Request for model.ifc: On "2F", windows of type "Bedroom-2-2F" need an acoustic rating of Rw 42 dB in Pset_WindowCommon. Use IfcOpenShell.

First a look at what the model holds.

```python
import ifcopenshell
import ifcopenshell.util.element

model = ifcopenshell.open("model.ifc")
print(model.schema)
storey = next(s for s in model.by_type("IfcBuildingStorey") if s.Name == "2F")
windows = [e for e in ifcopenshell.util.element.get_decomposition(storey) if e.is_a("IfcWindow")]
seen = {}
for e in windows:
    element_type = ifcopenshell.util.element.get_type(e)
    key = (element_type.Name if element_type != e and element_type else None, ifcopenshell.util.element.get_pset(e, "Pset_WindowCommon", "AcousticRating"))
    seen[key] = seen.get(key, 0) + 1
for (name, value), count in sorted(seen.items(), key=str):
    print(count, "x", name, "|", value)
```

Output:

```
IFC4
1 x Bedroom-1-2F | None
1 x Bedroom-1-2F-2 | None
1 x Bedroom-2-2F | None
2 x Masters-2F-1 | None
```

```python
import ifcopenshell
import ifcopenshell.api.pset
import ifcopenshell.util.element

model = ifcopenshell.open("model.ifc")

storey = next(s for s in model.by_type("IfcBuildingStorey") if s.Name == "2F")
windows = [e for e in ifcopenshell.util.element.get_decomposition(storey) if e.is_a("IfcWindow")]

count = 0
for e in windows:
    element_type = ifcopenshell.util.element.get_type(e)
    if element_type in (None, e) or element_type.Name != "Bedroom-2-2F":
        continue
    # add_pset returns the element's existing set when there is one.
    pset = ifcopenshell.api.pset.add_pset(model, product=e, name="Pset_WindowCommon")
    ifcopenshell.api.pset.edit_pset(model, pset=pset, properties={"AcousticRating": "Rw 42 dB"})
    count += 1

print(count, "windows updated")

model.write("model_v2.ifc")
```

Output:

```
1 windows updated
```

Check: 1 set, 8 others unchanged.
